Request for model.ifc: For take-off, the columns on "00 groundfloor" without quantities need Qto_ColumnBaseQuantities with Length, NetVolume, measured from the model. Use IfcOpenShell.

First a look at what the model holds.

```python
import ifcopenshell
import ifcopenshell.util.element
import ifcopenshell.util.unit

model = ifcopenshell.open("model.ifc")
print(model.schema)
for unit_type in ("LENGTHUNIT", "AREAUNIT", "VOLUMEUNIT"):
    print(unit_type, ifcopenshell.util.unit.calculate_unit_scale(model, unit_type))
storey = next(s for s in model.by_type("IfcBuildingStorey") if s.Name == "00 groundfloor")
columns = [e for e in ifcopenshell.util.element.get_decomposition(storey) if e.is_a("IfcColumn")]
for e in sorted(columns, key=lambda e: e.id()):
    print(e.id(), e.is_a(), e.Name, list(ifcopenshell.util.element.get_psets(e, qtos_only=True)), sep=" | ")
```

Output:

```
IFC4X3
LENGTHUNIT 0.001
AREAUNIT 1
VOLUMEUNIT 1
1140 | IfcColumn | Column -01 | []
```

```python
import ifcopenshell
import ifcopenshell.api.pset
import ifcopenshell.geom
import ifcopenshell.util.element
import ifcopenshell.util.shape
import ifcopenshell.util.unit

model = ifcopenshell.open("model.ifc")
unit_scale = ifcopenshell.util.unit.calculate_unit_scale(model)
volume_scale = ifcopenshell.util.unit.calculate_unit_scale(model, "VOLUMEUNIT")
settings = ifcopenshell.geom.settings()

storey = next(s for s in model.by_type("IfcBuildingStorey") if s.Name == "00 groundfloor")
columns = [e for e in ifcopenshell.util.element.get_decomposition(storey) if e.is_a("IfcColumn")]

for e in sorted(columns, key=lambda e: e.id()):
    if ifcopenshell.util.element.get_psets(e, qtos_only=True, should_inherit=False):
        continue
    # Geometry comes back in metres, in the element's own axes.
    shape = ifcopenshell.geom.create_shape(settings, e)
    values = {
        "Length": ifcopenshell.util.shape.get_z(shape.geometry) / unit_scale,
        "NetVolume": ifcopenshell.util.shape.get_volume(shape.geometry) / volume_scale,
    }
    qto = ifcopenshell.api.pset.add_qto(model, product=e, name="Qto_ColumnBaseQuantities")
    ifcopenshell.api.pset.edit_qto(model, qto=qto, properties=values)
    print(e.id(), {k: round(v, 3) for k, v in values.items()})

model.write("model_rev.ifc")
```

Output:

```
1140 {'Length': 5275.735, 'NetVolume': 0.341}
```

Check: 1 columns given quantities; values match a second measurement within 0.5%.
